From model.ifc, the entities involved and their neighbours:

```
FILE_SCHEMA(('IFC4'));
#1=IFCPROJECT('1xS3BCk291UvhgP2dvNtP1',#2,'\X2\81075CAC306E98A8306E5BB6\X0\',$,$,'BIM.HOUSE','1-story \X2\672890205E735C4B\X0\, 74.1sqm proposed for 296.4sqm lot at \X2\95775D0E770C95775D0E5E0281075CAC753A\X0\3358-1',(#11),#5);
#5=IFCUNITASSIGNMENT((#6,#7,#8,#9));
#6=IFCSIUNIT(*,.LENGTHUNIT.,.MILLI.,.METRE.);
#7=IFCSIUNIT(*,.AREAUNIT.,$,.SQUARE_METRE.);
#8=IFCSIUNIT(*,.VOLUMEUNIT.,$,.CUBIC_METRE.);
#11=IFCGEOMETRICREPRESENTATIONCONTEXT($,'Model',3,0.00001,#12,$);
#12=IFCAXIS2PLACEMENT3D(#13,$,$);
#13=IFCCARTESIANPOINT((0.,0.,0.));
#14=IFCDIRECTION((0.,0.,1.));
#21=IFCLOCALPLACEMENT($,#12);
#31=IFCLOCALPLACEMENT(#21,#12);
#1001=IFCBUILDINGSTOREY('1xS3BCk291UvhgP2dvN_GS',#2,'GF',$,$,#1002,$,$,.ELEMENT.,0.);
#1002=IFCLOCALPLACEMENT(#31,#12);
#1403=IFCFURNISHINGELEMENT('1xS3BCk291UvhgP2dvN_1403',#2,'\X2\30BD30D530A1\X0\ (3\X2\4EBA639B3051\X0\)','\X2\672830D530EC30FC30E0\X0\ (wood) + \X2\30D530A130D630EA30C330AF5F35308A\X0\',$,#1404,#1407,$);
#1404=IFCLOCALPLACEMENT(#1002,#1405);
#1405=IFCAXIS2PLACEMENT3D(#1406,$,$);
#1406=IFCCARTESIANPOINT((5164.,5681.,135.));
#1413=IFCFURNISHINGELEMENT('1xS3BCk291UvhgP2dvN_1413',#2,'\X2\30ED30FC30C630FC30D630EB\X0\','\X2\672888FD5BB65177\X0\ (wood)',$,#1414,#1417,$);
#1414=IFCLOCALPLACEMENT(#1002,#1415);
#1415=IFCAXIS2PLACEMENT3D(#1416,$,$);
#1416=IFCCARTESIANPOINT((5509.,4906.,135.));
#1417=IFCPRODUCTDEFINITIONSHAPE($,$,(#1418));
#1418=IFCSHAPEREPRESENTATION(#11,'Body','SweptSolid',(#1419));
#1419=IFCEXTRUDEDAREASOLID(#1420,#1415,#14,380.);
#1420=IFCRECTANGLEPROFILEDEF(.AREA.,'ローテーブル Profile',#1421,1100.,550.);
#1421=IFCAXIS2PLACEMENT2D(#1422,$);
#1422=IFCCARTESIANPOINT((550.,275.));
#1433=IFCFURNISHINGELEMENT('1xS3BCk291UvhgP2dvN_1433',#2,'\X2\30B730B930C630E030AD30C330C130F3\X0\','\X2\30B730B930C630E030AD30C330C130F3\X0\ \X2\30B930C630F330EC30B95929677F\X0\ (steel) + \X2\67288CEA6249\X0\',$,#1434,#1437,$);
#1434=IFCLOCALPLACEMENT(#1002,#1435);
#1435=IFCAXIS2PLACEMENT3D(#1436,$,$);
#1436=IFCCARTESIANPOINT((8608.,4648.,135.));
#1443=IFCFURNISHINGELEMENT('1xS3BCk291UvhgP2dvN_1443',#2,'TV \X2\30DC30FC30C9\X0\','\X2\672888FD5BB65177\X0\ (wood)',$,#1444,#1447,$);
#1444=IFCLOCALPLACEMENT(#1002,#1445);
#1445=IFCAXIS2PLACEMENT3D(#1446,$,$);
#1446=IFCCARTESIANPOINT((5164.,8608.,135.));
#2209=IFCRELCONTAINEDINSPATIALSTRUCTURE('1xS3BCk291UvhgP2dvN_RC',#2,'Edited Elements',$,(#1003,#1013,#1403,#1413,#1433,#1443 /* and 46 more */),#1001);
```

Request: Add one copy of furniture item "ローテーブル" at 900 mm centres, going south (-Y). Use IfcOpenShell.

```python
import numpy as np
import ifcopenshell
import ifcopenshell.api.geometry
import ifcopenshell.api.root
import ifcopenshell.util.element
import ifcopenshell.util.placement

model = ifcopenshell.open("model.ifc")


def reuse_history(source, copy):
    """copy_class also copies each property set's owner history, people and application; keep the originals."""
    for rel in copy.IsDefinedBy:
        if rel.is_a("IfcRelDefinesByProperties") and (history := rel.RelatingPropertyDefinition.OwnerHistory):
            rel.RelatingPropertyDefinition.OwnerHistory = source.OwnerHistory
            ifcopenshell.util.element.remove_deep2(model, history)


source = model.by_guid("1xS3BCk291UvhgP2dvN_1413")
base = ifcopenshell.util.placement.get_local_placement(source.ObjectPlacement)
step = np.array([0.0, -1.0, 0.0]) * 900.0

for i in range(1, 2):
    copy = ifcopenshell.api.root.copy_class(model, product=source)
    copy.Representation = ifcopenshell.util.element.copy_deep(
        model, source.Representation, exclude=["IfcGeometricRepresentationContext", "IfcRepresentationMap"]
    )
    reuse_history(source, copy)
    matrix = base.copy()
    matrix[:3, 3] += i * step
    print("added at", matrix[:3, 3].round(3) + 0.0)
    ifcopenshell.api.geometry.edit_object_placement(model, product=copy, matrix=matrix, is_si=False)

model.write("model_v2.ifc")
```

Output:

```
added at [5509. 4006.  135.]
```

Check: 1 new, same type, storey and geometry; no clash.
